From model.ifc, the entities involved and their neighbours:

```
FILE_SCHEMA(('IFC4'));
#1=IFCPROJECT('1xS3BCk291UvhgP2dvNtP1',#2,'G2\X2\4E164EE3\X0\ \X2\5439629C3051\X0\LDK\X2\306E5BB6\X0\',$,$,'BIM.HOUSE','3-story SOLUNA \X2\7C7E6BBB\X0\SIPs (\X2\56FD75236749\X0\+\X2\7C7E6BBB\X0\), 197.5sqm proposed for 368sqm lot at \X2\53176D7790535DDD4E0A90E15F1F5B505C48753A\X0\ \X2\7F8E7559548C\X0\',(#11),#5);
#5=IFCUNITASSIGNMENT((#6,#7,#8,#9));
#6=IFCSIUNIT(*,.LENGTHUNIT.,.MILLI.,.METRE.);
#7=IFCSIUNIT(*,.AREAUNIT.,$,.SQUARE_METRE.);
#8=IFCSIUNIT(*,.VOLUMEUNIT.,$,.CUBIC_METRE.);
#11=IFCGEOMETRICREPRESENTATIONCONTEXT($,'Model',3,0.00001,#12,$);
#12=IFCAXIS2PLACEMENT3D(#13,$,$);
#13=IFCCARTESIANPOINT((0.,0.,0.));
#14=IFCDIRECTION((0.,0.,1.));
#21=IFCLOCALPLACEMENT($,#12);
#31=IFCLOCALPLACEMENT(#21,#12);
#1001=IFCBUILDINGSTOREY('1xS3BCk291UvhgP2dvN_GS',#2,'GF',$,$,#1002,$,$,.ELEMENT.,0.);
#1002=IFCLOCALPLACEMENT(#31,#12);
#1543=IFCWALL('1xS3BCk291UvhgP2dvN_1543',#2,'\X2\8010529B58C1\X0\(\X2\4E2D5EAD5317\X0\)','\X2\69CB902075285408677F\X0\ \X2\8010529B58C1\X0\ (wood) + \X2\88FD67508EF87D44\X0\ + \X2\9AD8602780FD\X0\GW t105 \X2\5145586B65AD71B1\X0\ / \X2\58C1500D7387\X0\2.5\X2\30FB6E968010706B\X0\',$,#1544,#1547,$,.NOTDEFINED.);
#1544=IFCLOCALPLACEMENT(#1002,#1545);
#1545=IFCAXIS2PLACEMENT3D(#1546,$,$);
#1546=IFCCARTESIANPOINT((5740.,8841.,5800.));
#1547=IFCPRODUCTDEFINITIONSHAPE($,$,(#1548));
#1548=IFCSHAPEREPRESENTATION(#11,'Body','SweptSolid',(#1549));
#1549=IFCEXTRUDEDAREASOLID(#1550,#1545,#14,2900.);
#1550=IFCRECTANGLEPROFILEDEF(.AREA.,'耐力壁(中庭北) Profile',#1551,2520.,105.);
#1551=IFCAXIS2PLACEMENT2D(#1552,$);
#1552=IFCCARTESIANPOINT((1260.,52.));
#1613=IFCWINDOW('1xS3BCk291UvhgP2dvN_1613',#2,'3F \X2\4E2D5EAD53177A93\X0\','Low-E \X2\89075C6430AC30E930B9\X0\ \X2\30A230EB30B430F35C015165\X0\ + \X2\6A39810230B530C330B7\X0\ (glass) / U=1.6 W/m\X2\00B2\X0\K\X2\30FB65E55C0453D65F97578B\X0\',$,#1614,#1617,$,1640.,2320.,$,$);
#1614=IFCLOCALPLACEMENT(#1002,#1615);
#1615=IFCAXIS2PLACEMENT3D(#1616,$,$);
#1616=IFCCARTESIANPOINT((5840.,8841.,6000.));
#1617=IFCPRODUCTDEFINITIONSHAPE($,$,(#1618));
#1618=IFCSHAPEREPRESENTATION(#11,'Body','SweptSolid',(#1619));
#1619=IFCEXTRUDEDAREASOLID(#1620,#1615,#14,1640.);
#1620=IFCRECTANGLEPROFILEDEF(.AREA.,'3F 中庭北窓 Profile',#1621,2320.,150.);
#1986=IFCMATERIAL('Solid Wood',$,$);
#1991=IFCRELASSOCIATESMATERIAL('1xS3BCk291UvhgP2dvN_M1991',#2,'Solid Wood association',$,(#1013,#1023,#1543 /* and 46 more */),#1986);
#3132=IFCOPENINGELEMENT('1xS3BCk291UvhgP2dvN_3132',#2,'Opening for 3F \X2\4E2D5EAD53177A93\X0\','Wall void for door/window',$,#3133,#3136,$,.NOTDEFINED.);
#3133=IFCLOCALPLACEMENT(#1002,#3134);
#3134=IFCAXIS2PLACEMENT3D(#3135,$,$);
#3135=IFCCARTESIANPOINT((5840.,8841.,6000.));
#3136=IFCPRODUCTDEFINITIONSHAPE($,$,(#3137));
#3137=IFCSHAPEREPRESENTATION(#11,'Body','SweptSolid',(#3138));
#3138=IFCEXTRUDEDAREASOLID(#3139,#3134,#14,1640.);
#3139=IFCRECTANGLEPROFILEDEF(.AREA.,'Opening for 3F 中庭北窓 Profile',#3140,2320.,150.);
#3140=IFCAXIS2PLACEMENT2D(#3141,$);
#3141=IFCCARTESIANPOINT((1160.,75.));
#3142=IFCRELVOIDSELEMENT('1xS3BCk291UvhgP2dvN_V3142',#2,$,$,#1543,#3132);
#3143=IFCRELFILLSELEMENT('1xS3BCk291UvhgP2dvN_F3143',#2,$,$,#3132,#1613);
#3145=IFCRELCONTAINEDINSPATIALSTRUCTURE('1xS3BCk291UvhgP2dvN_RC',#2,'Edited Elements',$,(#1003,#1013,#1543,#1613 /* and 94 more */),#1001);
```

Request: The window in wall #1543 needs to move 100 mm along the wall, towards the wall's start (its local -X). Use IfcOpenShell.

```python
import ifcopenshell
import ifcopenshell.api.geometry
import ifcopenshell.util.placement

model = ifcopenshell.open("model.ifc")

window = model.by_guid("1xS3BCk291UvhgP2dvN_1613")
opening = window.FillsVoids[0].RelatingOpeningElement
wall = opening.VoidsElements[0].RelatingBuildingElement

wall_matrix = ifcopenshell.util.placement.get_local_placement(wall.ObjectPlacement)
shift = wall_matrix[:3, 0] * -100.0
before = ifcopenshell.util.placement.get_local_placement(window.ObjectPlacement)[:3, 3].copy()

# The window is not placed relative to its opening, so move both.
for product in (opening, window):
    matrix = ifcopenshell.util.placement.get_local_placement(product.ObjectPlacement)
    matrix[:3, 3] += shift
    ifcopenshell.api.geometry.edit_object_placement(model, product=product, matrix=matrix, is_si=False)

after = ifcopenshell.util.placement.get_local_placement(window.ObjectPlacement)[:3, 3]
print("window moved by", (after - before).round(3) + 0.0)

model.write("model_edited.ifc")
```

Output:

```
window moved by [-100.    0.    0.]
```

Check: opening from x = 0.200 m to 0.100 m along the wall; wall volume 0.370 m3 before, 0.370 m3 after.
